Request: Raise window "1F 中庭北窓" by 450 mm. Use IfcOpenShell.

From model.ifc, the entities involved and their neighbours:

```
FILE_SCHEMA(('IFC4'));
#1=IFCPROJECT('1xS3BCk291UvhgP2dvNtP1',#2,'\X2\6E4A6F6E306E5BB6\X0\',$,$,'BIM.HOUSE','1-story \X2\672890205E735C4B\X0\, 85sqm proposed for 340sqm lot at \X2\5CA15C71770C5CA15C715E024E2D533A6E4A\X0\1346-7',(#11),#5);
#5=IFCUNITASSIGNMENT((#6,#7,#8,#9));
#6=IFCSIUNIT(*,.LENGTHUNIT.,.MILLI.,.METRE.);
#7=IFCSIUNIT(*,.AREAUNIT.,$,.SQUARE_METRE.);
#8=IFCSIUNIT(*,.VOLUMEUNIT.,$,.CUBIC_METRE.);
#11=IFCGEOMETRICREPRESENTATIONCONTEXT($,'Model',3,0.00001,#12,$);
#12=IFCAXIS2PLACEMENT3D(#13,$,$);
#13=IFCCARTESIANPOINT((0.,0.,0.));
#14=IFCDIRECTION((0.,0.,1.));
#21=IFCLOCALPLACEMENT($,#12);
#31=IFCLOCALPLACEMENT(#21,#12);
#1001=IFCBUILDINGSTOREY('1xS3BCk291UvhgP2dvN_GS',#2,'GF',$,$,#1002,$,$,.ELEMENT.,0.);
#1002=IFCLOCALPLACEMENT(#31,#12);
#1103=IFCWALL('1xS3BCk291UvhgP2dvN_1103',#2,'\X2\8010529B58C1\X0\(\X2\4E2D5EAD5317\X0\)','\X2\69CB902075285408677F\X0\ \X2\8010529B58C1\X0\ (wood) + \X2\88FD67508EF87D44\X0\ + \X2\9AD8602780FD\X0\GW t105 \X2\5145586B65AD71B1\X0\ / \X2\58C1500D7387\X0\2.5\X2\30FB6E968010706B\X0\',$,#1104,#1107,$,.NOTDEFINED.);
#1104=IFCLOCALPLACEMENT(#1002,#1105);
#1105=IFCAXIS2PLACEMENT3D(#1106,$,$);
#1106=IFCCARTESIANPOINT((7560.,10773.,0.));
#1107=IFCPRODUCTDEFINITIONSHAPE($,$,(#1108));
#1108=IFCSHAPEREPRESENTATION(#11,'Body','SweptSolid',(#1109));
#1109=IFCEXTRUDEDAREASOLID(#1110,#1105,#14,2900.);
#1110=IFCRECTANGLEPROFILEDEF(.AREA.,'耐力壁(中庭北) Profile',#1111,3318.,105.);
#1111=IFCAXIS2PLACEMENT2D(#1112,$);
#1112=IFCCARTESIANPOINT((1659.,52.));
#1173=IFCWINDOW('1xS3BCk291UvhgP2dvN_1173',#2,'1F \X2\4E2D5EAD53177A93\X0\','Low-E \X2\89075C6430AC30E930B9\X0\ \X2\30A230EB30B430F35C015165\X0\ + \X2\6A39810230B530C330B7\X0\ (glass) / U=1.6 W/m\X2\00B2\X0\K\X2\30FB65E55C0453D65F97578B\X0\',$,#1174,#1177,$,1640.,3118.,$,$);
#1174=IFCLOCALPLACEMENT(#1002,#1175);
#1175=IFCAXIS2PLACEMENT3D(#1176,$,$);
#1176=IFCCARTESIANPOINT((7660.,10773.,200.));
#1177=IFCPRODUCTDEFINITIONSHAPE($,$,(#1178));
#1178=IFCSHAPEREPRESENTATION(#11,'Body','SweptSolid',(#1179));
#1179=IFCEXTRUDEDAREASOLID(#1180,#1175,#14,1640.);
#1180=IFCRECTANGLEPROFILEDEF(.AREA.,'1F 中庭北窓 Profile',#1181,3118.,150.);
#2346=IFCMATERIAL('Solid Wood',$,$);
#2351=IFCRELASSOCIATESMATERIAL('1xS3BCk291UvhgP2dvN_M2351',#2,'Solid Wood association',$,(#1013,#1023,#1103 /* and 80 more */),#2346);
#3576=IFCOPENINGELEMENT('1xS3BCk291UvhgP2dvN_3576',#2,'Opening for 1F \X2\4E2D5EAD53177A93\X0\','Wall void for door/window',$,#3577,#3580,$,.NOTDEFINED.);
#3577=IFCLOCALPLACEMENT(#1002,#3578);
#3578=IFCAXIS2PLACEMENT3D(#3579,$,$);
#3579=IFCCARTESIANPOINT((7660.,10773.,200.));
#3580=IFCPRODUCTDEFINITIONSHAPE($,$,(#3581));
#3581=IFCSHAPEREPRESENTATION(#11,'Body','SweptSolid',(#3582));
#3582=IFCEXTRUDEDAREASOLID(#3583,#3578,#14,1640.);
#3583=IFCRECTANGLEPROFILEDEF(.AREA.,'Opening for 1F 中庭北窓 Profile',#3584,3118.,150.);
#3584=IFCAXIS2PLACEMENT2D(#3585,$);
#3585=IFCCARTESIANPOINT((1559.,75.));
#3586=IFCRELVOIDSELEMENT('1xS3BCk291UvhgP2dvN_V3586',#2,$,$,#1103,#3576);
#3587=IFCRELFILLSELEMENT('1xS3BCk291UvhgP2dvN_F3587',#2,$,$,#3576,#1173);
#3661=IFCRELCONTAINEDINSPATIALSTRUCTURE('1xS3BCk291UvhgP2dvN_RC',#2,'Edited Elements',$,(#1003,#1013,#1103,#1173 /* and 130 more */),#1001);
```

```python
import numpy as np
import ifcopenshell
import ifcopenshell.api.geometry
import ifcopenshell.util.placement
import ifcopenshell.util.unit

model = ifcopenshell.open("model.ifc")
unit_scale = ifcopenshell.util.unit.calculate_unit_scale(model)

window = model.by_id(1173)
opening = window.FillsVoids[0].RelatingOpeningElement
dz = 0.45 / unit_scale

shift = np.array([0.0, 0.0, dz])
# The window is not placed relative to its opening, so move both.
for product in (opening, window):
    matrix = ifcopenshell.util.placement.get_local_placement(product.ObjectPlacement)
    matrix[:3, 3] += shift
    ifcopenshell.api.geometry.edit_object_placement(model, product=product, matrix=matrix, is_si=False)

print(f"moved by {dz * unit_scale:+.3f} m")

model.write("model_edited.ifc")
```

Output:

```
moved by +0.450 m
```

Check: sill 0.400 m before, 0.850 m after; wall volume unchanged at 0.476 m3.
